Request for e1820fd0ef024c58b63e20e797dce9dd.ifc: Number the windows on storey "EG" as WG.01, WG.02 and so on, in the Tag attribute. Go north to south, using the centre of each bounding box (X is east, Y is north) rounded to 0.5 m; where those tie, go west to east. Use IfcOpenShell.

First a look at what the model holds.

```python
import ifcopenshell
import ifcopenshell.util.element
import ifcopenshell.util.placement

model = ifcopenshell.open("e1820fd0ef024c58b63e20e797dce9dd.ifc")
print(model.schema)
storey = next(s for s in model.by_type("IfcBuildingStorey") if s.Name == "EG")
windows = [e for e in ifcopenshell.util.element.get_decomposition(storey) if e.is_a("IfcWindow")]
for e in sorted(windows, key=lambda e: e.id()):
    origin = ifcopenshell.util.placement.get_local_placement(e.ObjectPlacement)[:3, 3]
    print(e.id(), e.Tag, e.Name, origin.round(2) + 0.0, sep=" | ")
```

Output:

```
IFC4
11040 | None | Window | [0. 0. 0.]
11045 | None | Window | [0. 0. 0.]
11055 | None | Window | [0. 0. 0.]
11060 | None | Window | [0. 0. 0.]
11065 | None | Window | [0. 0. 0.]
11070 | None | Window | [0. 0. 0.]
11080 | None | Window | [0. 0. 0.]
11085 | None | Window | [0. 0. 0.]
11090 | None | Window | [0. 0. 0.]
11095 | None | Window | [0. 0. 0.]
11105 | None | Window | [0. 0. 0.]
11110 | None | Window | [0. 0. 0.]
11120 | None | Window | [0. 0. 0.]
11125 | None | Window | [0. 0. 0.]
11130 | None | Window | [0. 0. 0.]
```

```python
import ifcopenshell
import ifcopenshell.geom
import ifcopenshell.util.element
import ifcopenshell.util.shape

model = ifcopenshell.open("e1820fd0ef024c58b63e20e797dce9dd.ifc")
settings = ifcopenshell.geom.settings()
settings.set("use-world-coords", True)


def centre(element):
    shape = ifcopenshell.geom.create_shape(settings, element)
    return ifcopenshell.util.shape.get_bbox_centroid(shape.geometry)


storey = next(s for s in model.by_type("IfcBuildingStorey") if s.Name == "EG")
windows = [e for e in ifcopenshell.util.element.get_decomposition(storey) if e.is_a("IfcWindow")]

# Insertion points can sit at a corner or the storey origin, so sort by the geometry (in metres).
centres = {e: centre(e) for e in windows}
windows.sort(key=lambda e: (-round(centres[e][1] / 0.5), centres[e][0]))

for i, e in enumerate(windows, start=1):
    number = f"WG.{i:02d}"
    e.Tag = number
    print(e.id(), number)

model.write("e1820fd0ef024c58b63e20e797dce9dd-out.ifc")
```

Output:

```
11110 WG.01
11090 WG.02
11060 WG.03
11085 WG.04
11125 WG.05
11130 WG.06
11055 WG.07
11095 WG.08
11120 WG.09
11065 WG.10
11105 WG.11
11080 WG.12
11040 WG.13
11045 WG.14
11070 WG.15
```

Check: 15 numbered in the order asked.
